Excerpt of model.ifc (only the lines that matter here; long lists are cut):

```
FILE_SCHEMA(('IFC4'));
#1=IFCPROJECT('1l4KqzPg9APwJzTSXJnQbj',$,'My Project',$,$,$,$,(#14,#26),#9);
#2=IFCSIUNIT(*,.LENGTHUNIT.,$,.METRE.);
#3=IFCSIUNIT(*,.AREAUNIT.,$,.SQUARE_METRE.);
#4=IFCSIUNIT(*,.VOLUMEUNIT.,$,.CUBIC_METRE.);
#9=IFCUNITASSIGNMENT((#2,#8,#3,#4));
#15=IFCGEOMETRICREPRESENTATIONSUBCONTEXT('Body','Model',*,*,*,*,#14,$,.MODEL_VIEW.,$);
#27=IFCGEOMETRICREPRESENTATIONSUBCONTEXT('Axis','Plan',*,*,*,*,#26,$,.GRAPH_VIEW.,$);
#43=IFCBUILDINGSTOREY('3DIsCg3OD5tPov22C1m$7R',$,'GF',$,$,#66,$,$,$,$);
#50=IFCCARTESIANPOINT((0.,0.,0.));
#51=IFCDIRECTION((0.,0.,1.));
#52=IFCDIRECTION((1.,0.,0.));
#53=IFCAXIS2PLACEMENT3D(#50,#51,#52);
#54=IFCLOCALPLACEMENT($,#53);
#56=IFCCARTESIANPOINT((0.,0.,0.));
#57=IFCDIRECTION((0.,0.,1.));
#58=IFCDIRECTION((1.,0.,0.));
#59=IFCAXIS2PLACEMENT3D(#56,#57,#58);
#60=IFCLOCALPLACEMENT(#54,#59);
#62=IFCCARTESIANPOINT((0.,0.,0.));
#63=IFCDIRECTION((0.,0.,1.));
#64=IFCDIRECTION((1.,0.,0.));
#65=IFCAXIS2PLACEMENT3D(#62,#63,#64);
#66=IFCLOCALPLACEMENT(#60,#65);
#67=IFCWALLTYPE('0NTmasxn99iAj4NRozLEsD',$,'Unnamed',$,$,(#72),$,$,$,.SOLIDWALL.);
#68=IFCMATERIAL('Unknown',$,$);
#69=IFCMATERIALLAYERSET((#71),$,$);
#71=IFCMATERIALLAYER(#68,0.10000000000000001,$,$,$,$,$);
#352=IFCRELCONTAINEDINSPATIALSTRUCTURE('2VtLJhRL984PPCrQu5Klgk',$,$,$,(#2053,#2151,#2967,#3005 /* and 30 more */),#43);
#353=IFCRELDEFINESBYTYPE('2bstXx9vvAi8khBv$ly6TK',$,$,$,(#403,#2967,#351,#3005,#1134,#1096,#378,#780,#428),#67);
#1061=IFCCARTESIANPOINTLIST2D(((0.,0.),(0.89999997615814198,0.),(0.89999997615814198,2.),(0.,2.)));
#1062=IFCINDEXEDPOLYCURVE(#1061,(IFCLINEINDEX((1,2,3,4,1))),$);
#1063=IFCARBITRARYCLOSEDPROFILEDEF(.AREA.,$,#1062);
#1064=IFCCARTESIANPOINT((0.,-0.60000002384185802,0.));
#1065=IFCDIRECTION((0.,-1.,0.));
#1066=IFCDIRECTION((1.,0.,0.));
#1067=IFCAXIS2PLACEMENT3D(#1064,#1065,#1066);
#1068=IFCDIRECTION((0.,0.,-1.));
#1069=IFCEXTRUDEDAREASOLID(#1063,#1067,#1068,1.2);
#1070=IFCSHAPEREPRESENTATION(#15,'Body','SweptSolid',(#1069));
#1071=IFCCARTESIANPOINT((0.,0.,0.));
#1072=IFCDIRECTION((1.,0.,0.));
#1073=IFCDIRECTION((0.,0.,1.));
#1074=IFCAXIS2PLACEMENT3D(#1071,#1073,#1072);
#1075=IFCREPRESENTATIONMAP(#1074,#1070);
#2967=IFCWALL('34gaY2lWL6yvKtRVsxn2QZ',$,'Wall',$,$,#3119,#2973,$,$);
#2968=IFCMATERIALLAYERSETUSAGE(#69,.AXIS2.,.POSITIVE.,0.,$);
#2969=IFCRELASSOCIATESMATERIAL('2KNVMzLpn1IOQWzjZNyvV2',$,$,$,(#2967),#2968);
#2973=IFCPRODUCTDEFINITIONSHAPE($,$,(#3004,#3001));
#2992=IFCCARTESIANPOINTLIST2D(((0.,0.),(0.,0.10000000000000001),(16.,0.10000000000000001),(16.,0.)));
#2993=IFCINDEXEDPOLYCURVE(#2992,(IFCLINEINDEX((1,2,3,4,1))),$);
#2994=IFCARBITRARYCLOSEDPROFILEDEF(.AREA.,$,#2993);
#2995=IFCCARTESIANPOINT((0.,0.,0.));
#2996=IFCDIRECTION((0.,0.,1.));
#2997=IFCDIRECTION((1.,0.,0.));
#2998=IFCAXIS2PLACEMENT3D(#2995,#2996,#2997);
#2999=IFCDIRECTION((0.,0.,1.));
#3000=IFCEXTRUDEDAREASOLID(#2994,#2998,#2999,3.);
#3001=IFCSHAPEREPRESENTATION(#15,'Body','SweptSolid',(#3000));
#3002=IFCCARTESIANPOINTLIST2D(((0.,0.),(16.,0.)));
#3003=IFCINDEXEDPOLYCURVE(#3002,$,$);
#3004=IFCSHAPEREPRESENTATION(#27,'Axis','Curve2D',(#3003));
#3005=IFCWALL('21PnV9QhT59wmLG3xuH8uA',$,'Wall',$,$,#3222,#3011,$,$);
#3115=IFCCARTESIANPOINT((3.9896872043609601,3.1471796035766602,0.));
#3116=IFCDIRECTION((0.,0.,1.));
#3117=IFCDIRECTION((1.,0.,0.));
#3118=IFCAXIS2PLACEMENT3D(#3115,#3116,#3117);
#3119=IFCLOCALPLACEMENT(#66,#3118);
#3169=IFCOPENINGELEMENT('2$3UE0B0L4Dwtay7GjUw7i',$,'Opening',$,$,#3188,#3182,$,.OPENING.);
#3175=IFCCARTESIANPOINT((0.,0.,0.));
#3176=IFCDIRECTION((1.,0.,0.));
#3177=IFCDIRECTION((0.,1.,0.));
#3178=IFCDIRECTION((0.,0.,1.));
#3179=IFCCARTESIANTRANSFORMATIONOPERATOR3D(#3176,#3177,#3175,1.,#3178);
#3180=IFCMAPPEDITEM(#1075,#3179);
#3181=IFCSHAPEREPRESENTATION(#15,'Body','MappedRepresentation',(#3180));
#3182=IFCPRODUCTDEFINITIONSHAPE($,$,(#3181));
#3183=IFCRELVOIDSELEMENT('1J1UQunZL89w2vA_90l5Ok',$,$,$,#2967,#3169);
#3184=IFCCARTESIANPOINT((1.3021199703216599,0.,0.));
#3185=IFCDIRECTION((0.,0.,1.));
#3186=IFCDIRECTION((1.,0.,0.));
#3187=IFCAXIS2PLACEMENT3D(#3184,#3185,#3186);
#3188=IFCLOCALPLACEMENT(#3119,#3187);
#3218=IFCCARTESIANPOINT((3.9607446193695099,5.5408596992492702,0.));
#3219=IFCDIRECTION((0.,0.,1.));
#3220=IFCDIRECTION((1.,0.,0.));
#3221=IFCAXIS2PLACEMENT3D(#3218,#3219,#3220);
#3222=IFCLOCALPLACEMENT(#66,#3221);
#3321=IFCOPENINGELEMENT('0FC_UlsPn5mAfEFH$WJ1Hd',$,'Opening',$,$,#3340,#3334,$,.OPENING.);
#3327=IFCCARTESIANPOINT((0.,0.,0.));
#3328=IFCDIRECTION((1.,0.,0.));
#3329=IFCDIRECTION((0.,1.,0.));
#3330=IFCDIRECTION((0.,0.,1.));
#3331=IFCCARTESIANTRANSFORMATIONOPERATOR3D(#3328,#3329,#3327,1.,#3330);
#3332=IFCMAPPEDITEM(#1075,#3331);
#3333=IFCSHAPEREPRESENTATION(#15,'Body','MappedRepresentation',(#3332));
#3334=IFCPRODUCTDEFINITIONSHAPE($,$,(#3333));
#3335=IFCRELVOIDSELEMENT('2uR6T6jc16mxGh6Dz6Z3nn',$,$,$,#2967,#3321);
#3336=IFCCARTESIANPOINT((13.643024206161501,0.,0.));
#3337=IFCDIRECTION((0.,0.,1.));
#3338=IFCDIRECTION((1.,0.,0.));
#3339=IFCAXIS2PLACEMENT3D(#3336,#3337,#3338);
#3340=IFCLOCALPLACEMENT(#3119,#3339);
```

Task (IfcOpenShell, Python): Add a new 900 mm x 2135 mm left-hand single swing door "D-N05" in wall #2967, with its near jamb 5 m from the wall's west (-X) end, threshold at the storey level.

```python
import numpy as np
import ifcopenshell
import ifcopenshell.api.feature
import ifcopenshell.api.geometry
import ifcopenshell.api.root
import ifcopenshell.api.spatial
import ifcopenshell.geom
import ifcopenshell.util.element
import ifcopenshell.util.placement
import ifcopenshell.util.representation
import ifcopenshell.util.shape
import ifcopenshell.util.unit

model = ifcopenshell.open("model.ifc")
unit_scale = ifcopenshell.util.unit.calculate_unit_scale(model)
settings = ifcopenshell.geom.settings()


def volume(element):
    """Net volume in cubic metres, openings subtracted."""
    shape = ifcopenshell.geom.create_shape(settings, element)
    return ifcopenshell.util.shape.get_volume(shape.geometry)


wall = model.by_guid("34gaY2lWL6yvKtRVsxn2QZ")
storey = ifcopenshell.util.element.get_container(wall, ifc_class="IfcBuildingStorey")
context = ifcopenshell.util.representation.get_context(model, "Model", "Body", "MODEL_VIEW")
before = volume(wall)

width, height, from_end, sill = 0.9, 2.135, 5, 0.0  # metres

# The wall runs along its own X axis, and the end named is its -X end.
wall_shape = ifcopenshell.geom.create_shape(settings, wall)
x, y, z = ifcopenshell.util.shape.get_vertices(wall_shape.geometry).T
start = x.min() + from_end
face, thickness = float(y.min()), float(y.max() - y.min())
wall_matrix = ifcopenshell.util.placement.get_local_placement(wall.ObjectPlacement)
level = ifcopenshell.util.placement.get_local_placement(storey.ObjectPlacement)[2, 3]


def in_wall(x, y):
    """Placement at x, y metres in the wall's axes, at sill height."""
    matrix = wall_matrix.copy()
    matrix[:, 3] = wall_matrix @ np.array([x / unit_scale, y / unit_scale, 0.0, 1.0])
    matrix[2, 3] = level + sill / unit_scale
    return matrix


# Opening: a box that overshoots both wall faces by 50 mm.
opening = ifcopenshell.api.root.create_entity(model, ifc_class="IfcOpeningElement", predefined_type="OPENING")
box = ifcopenshell.api.geometry.add_wall_representation(
    model, context=context, length=width, height=height, thickness=thickness + 0.1
)
ifcopenshell.api.geometry.assign_representation(model, product=opening, representation=box)
ifcopenshell.api.geometry.edit_object_placement(model, product=opening, matrix=in_wall(start, face - 0.05), is_si=False)
ifcopenshell.api.feature.add_feature(model, feature=opening, element=wall)

door = ifcopenshell.api.root.create_entity(model, ifc_class="IfcDoor", name="D-N05", predefined_type="DOOR")
door.OverallWidth, door.OverallHeight = width / unit_scale, height / unit_scale
door.OperationType = "SINGLE_SWING_LEFT"
body = ifcopenshell.api.geometry.add_door_representation(
    model,
    context=context,
    overall_width=door.OverallWidth,
    overall_height=door.OverallHeight,
    operation_type="SINGLE_SWING_LEFT",
    lining_properties={"LiningDepth": thickness / unit_scale, "ThresholdDepth": thickness / unit_scale},
)
ifcopenshell.api.geometry.assign_representation(model, product=door, representation=body)
ifcopenshell.api.spatial.assign_container(model, products=[door], relating_structure=storey)
ifcopenshell.api.feature.add_filling(model, opening=opening, element=door)

# The lining spans the wall, so the door starts at the wall face.
ifcopenshell.api.geometry.edit_object_placement(model, product=door, matrix=in_wall(start, face), is_si=False)

after = volume(wall)

print(f"wall volume {before:.3f} -> {after:.3f} m3")

model.write("model_updated.ifc")
```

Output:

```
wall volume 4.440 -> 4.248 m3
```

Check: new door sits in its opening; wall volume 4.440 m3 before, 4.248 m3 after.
